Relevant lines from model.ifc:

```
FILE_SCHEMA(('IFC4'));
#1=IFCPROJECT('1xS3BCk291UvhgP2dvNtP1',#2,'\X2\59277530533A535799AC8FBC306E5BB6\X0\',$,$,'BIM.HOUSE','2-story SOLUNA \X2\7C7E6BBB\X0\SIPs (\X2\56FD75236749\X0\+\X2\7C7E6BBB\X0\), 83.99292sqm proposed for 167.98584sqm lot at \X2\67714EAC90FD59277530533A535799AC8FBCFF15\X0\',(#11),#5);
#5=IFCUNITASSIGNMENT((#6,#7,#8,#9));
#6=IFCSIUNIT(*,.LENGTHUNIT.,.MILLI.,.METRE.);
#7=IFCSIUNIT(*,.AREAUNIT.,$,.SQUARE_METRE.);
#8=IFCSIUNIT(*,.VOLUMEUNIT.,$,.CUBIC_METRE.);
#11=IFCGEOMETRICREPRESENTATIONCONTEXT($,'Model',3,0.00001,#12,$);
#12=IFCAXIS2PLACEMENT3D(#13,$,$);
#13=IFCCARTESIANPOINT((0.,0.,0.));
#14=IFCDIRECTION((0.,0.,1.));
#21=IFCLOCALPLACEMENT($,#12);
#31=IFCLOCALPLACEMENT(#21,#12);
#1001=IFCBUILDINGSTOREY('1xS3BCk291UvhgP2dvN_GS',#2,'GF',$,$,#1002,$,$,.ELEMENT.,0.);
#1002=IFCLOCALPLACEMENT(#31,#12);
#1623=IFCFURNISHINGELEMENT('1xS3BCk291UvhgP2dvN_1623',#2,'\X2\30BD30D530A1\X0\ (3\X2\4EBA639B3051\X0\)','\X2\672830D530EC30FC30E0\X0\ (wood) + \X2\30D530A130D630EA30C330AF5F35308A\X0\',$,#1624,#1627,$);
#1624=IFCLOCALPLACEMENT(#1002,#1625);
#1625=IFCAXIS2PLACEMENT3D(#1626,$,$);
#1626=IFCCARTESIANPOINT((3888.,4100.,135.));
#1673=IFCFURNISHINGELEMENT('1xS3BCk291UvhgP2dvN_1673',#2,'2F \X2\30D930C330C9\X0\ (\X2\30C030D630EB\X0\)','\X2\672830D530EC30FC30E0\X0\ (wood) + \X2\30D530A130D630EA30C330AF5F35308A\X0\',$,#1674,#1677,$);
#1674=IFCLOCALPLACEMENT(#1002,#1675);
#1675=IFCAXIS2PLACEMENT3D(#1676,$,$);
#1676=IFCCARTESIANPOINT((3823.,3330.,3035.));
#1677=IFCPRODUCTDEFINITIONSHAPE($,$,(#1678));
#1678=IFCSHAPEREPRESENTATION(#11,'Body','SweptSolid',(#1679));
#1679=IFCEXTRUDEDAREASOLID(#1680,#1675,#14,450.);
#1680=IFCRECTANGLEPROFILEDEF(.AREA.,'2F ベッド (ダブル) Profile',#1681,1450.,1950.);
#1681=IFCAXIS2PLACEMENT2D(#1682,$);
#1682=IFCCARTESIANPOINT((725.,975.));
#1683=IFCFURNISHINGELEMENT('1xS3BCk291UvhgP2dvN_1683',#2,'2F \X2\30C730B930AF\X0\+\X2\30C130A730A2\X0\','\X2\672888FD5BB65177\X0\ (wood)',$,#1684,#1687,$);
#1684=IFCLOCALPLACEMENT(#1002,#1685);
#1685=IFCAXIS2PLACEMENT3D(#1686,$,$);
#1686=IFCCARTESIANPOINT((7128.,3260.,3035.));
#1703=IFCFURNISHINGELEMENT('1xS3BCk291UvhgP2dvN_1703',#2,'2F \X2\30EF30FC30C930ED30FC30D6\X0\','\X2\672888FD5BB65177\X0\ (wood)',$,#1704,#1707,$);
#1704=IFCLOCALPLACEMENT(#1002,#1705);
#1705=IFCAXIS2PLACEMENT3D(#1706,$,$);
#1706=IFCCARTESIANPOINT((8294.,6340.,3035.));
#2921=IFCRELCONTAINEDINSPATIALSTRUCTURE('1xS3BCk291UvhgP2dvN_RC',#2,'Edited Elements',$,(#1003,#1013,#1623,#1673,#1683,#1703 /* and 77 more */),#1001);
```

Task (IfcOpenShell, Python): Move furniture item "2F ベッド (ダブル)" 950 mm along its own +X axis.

```python
import ifcopenshell
import ifcopenshell.api.geometry
import ifcopenshell.util.placement
import ifcopenshell.util.unit

model = ifcopenshell.open("model.ifc")
unit_scale = ifcopenshell.util.unit.calculate_unit_scale(model)

item = model.by_id(1673)
matrix = ifcopenshell.util.placement.get_local_placement(item.ObjectPlacement)
matrix[:3, 3] += matrix[:3, 0] * 0.95 / unit_scale
ifcopenshell.api.geometry.edit_object_placement(model, product=item, matrix=matrix, is_si=False)

print(ifcopenshell.util.placement.get_local_placement(item.ObjectPlacement).round(3) + 0.0)

model.write("model_edited.ifc")
```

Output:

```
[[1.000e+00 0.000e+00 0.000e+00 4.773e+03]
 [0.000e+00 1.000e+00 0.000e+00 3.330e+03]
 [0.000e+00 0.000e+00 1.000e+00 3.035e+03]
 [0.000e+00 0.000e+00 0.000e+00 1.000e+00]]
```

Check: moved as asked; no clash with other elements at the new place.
